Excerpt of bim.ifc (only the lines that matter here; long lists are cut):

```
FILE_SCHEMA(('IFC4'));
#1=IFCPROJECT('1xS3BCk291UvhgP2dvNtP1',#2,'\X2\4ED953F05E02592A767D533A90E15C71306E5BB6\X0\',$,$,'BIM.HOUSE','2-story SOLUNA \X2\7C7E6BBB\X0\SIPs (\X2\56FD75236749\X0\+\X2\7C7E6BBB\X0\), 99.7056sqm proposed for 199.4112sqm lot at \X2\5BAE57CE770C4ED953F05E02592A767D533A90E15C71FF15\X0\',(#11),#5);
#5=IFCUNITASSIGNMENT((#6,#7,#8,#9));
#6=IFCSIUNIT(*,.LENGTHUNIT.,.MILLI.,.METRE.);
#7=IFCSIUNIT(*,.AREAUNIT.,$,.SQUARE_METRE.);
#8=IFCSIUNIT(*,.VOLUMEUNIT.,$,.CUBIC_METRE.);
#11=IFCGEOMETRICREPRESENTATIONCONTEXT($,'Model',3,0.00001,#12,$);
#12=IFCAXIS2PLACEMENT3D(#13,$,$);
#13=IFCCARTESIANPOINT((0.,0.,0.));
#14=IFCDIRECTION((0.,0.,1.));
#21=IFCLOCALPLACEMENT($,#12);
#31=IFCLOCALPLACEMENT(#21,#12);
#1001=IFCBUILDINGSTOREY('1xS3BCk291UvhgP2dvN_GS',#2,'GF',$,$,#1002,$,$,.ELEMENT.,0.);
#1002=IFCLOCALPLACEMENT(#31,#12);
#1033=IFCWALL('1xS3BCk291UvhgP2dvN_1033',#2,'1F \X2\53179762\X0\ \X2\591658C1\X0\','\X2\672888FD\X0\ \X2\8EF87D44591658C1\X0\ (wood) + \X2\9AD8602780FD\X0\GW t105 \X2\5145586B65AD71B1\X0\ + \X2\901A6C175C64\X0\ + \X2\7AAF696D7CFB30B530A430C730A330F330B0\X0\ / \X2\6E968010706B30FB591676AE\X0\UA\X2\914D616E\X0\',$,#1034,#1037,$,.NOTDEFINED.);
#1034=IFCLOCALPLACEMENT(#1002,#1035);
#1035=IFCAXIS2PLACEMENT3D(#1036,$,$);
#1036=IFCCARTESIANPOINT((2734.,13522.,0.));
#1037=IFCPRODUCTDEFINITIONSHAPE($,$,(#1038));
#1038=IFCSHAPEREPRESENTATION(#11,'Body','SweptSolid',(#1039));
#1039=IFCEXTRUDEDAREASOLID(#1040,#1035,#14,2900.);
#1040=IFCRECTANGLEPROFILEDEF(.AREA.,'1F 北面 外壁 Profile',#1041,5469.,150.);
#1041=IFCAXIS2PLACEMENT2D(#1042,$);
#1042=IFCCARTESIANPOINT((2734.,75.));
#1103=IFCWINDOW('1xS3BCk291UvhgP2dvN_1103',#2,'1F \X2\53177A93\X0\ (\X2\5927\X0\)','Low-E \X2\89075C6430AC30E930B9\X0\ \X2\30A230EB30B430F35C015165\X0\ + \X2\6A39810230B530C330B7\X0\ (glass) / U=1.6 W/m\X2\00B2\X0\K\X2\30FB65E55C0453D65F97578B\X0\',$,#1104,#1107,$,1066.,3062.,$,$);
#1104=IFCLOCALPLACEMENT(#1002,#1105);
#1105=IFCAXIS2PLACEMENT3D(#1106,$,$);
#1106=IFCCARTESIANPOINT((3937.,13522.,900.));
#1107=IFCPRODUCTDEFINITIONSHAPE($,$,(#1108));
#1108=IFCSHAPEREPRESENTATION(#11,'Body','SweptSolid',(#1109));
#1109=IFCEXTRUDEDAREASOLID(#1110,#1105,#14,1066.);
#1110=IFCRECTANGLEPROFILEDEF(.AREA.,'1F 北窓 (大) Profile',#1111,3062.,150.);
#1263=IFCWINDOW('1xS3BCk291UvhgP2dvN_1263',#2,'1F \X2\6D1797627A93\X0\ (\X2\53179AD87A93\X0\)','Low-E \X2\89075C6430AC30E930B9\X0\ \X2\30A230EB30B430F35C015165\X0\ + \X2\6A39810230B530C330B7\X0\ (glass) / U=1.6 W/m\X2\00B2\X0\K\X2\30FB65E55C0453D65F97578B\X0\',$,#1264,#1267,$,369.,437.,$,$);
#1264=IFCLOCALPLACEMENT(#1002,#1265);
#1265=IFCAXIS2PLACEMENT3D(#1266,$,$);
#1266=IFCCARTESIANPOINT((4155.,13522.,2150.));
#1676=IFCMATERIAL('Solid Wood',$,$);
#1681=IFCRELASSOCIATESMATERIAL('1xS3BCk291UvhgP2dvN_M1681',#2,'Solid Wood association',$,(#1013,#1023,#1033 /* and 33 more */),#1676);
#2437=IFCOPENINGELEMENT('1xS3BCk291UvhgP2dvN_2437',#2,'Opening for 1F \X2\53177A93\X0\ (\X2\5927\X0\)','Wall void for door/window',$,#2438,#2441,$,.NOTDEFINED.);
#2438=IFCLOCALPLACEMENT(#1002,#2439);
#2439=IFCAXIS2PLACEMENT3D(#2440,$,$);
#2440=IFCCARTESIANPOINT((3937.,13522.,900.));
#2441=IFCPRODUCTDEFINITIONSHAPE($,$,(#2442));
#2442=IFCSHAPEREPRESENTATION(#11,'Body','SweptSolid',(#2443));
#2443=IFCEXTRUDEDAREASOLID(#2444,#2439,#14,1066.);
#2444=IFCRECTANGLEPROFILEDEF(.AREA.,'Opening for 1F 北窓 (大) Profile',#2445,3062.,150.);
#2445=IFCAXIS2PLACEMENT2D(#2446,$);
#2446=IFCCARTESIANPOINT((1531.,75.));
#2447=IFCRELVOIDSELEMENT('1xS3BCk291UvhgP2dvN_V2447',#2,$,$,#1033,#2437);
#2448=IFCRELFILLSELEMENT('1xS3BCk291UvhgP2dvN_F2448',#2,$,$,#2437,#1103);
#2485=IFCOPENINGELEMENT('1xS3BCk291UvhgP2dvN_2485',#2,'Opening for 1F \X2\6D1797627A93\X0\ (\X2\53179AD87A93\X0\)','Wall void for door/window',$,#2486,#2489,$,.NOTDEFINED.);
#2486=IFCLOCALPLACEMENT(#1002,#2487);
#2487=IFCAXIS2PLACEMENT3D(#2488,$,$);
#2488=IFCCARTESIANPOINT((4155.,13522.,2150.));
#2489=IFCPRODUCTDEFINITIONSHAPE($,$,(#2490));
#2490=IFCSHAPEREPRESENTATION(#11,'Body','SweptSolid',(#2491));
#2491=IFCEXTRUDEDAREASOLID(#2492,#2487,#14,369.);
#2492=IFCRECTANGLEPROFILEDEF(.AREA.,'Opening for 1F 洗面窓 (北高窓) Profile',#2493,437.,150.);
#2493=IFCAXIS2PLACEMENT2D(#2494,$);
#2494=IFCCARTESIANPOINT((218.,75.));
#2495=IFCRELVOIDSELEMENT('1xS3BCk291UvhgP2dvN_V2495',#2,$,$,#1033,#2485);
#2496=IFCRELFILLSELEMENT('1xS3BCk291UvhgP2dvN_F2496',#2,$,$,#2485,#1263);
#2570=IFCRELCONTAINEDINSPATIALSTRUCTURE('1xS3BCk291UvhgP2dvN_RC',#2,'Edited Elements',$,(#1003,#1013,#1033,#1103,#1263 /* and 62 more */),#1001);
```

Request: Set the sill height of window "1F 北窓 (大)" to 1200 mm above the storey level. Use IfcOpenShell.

```python
import numpy as np
import ifcopenshell
import ifcopenshell.api.geometry
import ifcopenshell.geom
import ifcopenshell.util.element
import ifcopenshell.util.placement
import ifcopenshell.util.shape
import ifcopenshell.util.unit

model = ifcopenshell.open("bim.ifc")
unit_scale = ifcopenshell.util.unit.calculate_unit_scale(model)

window = model.by_id(1103)
opening = window.FillsVoids[0].RelatingOpeningElement
storey = ifcopenshell.util.element.get_container(window, ifc_class="IfcBuildingStorey")
level = ifcopenshell.util.placement.get_local_placement(storey.ObjectPlacement)[2, 3]

# The opening's origin need not be at the sill, so measure its lowest point.
shape = ifcopenshell.geom.create_shape(ifcopenshell.geom.settings(), opening)
bottom = ifcopenshell.util.shape.get_shape_bottom_elevation(shape, shape.geometry) / unit_scale
dz = level + 1200.0 - bottom

shift = np.array([0.0, 0.0, dz])
# The window is not placed relative to its opening, so move both.
for product in (opening, window):
    matrix = ifcopenshell.util.placement.get_local_placement(product.ObjectPlacement)
    matrix[:3, 3] += shift
    ifcopenshell.api.geometry.edit_object_placement(model, product=product, matrix=matrix, is_si=False)

print(f"moved by {dz * unit_scale:+.3f} m")

model.write("bim_rev.ifc")
```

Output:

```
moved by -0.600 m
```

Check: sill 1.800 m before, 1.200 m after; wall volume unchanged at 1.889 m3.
